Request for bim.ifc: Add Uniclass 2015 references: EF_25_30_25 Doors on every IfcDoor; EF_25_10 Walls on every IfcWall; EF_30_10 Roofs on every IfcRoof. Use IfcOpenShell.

First a look at what the model holds.

```python
import ifcopenshell

model = ifcopenshell.open("bim.ifc")
print(model.schema)
print("classifications:", [c.Name for c in model.by_type("IfcClassification")])
for ifc_class in ("IfcDoor", "IfcRoof", "IfcStair", "IfcWall", "IfcWindow"):
    print(ifc_class, len(model.by_type(ifc_class)))
```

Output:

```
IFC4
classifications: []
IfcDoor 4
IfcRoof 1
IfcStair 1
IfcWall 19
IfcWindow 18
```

```python
import ifcopenshell
import ifcopenshell.api.classification

model = ifcopenshell.open("bim.ifc")

system = ifcopenshell.api.classification.add_classification(model, classification="Uniclass 2015")

codes = {
    "IfcDoor": ("EF_25_30_25", "Doors"),
    "IfcWall": ("EF_25_10", "Walls"),
    "IfcRoof": ("EF_30_10", "Roofs"),
}
for ifc_class, (code, name) in codes.items():
    products = model.by_type(ifc_class)
    ifcopenshell.api.classification.add_reference(
        model, products=products, classification=system, identification=code, name=name
    )
    print(code, len(products))

model.write("bim_v2.ifc")
```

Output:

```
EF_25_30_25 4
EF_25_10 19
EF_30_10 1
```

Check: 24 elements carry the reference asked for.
